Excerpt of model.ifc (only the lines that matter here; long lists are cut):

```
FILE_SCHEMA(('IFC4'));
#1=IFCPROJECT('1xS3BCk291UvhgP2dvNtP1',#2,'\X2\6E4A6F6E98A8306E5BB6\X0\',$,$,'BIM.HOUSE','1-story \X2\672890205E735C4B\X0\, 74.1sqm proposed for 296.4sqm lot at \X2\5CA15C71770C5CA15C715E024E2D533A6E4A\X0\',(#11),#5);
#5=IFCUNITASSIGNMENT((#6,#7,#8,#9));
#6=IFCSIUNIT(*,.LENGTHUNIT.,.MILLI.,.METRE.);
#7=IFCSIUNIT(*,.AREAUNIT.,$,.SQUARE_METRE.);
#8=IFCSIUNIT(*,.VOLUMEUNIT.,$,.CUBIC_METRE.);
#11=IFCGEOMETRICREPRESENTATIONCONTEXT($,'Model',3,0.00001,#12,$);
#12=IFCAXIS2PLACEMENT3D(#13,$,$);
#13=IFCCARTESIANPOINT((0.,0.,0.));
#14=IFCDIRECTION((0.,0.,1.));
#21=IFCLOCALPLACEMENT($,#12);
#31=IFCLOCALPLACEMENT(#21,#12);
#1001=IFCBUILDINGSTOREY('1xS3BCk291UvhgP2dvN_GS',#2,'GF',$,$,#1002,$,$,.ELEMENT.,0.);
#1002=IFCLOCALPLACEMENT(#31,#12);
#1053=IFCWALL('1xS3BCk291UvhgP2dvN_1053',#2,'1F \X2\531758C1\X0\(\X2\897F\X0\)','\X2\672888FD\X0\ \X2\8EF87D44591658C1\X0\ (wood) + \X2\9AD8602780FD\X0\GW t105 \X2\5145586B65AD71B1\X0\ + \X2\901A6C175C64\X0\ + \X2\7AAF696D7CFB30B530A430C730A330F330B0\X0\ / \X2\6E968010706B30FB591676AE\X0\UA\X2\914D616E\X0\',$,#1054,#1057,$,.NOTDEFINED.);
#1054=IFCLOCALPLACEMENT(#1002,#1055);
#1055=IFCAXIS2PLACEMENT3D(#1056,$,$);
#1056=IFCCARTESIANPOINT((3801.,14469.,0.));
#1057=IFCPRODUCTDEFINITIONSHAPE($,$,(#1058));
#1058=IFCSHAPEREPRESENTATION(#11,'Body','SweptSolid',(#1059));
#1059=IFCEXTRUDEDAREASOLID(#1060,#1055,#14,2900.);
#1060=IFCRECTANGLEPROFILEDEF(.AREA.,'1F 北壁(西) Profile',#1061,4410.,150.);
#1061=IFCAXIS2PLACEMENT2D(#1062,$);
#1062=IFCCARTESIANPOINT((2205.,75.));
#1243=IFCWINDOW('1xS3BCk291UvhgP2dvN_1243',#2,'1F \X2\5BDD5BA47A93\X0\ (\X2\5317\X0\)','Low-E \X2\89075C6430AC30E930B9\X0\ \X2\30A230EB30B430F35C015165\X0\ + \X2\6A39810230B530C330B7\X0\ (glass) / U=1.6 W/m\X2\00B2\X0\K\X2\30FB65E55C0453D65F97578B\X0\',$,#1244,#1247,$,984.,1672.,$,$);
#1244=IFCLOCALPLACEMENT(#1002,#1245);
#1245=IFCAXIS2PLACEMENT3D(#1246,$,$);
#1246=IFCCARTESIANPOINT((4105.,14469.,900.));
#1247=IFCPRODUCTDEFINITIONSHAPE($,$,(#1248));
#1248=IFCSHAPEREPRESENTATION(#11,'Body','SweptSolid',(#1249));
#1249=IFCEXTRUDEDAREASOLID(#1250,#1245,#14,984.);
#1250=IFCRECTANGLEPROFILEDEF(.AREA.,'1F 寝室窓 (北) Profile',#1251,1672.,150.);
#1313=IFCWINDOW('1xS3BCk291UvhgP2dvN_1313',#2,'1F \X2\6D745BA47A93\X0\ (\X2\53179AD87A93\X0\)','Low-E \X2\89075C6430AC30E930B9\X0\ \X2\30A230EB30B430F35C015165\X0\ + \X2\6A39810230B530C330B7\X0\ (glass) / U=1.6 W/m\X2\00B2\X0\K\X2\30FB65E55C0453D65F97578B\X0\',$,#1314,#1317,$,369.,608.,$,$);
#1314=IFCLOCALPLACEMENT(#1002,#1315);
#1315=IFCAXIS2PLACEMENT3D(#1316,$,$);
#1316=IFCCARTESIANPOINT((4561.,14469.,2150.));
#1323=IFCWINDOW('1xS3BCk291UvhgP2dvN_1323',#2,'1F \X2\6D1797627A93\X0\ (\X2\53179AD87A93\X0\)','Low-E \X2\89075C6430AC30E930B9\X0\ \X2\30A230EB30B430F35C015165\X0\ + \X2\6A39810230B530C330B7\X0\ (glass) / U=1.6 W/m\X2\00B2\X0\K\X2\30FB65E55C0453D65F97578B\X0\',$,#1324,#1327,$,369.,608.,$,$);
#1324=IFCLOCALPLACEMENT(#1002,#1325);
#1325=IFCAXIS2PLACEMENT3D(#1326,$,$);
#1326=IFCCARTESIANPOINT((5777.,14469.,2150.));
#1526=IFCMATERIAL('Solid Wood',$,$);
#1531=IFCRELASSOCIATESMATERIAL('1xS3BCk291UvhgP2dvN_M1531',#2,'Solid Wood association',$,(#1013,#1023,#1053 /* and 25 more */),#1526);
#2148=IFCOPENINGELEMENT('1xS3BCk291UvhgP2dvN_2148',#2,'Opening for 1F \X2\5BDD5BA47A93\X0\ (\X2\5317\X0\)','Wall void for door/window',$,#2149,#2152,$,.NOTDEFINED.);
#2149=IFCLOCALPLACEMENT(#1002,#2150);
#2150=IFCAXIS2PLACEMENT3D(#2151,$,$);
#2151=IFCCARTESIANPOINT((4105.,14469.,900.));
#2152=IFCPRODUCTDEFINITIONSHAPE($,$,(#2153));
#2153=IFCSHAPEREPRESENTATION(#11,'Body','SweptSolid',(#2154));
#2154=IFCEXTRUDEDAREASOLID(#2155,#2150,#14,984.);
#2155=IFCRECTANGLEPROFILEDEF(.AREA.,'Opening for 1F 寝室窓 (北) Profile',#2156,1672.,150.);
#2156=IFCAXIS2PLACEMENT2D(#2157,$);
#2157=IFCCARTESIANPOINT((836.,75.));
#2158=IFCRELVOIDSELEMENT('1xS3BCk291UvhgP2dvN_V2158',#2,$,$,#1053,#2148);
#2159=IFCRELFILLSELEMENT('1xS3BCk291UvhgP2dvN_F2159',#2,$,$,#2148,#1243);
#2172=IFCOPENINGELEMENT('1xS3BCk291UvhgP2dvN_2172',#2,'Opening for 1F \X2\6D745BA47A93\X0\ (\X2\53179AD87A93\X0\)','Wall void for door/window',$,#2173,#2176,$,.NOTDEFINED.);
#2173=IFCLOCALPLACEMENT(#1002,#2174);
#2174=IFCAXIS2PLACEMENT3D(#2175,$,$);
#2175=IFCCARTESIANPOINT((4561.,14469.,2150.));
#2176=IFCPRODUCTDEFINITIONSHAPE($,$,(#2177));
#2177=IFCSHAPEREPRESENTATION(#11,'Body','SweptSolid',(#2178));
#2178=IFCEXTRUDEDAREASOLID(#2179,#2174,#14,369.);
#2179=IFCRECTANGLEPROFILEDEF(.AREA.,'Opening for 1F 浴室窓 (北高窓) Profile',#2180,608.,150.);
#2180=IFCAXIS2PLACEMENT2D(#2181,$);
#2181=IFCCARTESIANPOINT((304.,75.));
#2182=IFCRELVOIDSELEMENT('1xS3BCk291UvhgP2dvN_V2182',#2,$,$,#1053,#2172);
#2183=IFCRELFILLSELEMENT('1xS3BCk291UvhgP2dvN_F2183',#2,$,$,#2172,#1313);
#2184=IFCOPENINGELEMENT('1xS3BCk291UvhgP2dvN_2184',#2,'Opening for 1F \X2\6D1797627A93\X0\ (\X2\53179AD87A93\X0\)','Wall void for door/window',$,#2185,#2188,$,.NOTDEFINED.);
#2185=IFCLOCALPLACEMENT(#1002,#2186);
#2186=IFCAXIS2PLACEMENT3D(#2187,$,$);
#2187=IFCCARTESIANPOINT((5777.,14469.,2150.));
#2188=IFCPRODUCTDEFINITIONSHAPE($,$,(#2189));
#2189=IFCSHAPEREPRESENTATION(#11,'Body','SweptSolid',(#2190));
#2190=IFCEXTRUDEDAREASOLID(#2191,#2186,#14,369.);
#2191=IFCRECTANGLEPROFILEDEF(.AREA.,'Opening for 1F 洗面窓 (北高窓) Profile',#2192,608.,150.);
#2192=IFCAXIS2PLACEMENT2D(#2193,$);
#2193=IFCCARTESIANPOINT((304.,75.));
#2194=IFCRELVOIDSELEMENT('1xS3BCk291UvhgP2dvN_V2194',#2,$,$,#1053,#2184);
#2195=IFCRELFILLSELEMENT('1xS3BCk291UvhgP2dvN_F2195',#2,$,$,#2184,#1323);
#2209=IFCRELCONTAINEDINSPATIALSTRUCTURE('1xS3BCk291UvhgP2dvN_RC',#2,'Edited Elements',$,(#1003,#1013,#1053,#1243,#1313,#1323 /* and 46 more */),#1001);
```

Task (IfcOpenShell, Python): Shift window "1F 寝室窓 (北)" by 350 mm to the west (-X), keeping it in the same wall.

```python
import ifcopenshell
import ifcopenshell.api.geometry
import ifcopenshell.util.placement
import ifcopenshell.util.unit

model = ifcopenshell.open("model.ifc")
unit_scale = ifcopenshell.util.unit.calculate_unit_scale(model)

window = model.by_guid("1xS3BCk291UvhgP2dvN_1243")
opening = window.FillsVoids[0].RelatingOpeningElement
wall = opening.VoidsElements[0].RelatingBuildingElement

wall_matrix = ifcopenshell.util.placement.get_local_placement(wall.ObjectPlacement)
shift = wall_matrix[:3, 0] * -0.35 / unit_scale
before = ifcopenshell.util.placement.get_local_placement(window.ObjectPlacement)[:3, 3].copy()

# The window is not placed relative to its opening, so move both.
for product in (opening, window):
    matrix = ifcopenshell.util.placement.get_local_placement(product.ObjectPlacement)
    matrix[:3, 3] += shift
    ifcopenshell.api.geometry.edit_object_placement(model, product=product, matrix=matrix, is_si=False)

after = ifcopenshell.util.placement.get_local_placement(window.ObjectPlacement)[:3, 3]
print("window moved by", (after - before).round(3) + 0.0)

model.write("model_updated.ifc")
```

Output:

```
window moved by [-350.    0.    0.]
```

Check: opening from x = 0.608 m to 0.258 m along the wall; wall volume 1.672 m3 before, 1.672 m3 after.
